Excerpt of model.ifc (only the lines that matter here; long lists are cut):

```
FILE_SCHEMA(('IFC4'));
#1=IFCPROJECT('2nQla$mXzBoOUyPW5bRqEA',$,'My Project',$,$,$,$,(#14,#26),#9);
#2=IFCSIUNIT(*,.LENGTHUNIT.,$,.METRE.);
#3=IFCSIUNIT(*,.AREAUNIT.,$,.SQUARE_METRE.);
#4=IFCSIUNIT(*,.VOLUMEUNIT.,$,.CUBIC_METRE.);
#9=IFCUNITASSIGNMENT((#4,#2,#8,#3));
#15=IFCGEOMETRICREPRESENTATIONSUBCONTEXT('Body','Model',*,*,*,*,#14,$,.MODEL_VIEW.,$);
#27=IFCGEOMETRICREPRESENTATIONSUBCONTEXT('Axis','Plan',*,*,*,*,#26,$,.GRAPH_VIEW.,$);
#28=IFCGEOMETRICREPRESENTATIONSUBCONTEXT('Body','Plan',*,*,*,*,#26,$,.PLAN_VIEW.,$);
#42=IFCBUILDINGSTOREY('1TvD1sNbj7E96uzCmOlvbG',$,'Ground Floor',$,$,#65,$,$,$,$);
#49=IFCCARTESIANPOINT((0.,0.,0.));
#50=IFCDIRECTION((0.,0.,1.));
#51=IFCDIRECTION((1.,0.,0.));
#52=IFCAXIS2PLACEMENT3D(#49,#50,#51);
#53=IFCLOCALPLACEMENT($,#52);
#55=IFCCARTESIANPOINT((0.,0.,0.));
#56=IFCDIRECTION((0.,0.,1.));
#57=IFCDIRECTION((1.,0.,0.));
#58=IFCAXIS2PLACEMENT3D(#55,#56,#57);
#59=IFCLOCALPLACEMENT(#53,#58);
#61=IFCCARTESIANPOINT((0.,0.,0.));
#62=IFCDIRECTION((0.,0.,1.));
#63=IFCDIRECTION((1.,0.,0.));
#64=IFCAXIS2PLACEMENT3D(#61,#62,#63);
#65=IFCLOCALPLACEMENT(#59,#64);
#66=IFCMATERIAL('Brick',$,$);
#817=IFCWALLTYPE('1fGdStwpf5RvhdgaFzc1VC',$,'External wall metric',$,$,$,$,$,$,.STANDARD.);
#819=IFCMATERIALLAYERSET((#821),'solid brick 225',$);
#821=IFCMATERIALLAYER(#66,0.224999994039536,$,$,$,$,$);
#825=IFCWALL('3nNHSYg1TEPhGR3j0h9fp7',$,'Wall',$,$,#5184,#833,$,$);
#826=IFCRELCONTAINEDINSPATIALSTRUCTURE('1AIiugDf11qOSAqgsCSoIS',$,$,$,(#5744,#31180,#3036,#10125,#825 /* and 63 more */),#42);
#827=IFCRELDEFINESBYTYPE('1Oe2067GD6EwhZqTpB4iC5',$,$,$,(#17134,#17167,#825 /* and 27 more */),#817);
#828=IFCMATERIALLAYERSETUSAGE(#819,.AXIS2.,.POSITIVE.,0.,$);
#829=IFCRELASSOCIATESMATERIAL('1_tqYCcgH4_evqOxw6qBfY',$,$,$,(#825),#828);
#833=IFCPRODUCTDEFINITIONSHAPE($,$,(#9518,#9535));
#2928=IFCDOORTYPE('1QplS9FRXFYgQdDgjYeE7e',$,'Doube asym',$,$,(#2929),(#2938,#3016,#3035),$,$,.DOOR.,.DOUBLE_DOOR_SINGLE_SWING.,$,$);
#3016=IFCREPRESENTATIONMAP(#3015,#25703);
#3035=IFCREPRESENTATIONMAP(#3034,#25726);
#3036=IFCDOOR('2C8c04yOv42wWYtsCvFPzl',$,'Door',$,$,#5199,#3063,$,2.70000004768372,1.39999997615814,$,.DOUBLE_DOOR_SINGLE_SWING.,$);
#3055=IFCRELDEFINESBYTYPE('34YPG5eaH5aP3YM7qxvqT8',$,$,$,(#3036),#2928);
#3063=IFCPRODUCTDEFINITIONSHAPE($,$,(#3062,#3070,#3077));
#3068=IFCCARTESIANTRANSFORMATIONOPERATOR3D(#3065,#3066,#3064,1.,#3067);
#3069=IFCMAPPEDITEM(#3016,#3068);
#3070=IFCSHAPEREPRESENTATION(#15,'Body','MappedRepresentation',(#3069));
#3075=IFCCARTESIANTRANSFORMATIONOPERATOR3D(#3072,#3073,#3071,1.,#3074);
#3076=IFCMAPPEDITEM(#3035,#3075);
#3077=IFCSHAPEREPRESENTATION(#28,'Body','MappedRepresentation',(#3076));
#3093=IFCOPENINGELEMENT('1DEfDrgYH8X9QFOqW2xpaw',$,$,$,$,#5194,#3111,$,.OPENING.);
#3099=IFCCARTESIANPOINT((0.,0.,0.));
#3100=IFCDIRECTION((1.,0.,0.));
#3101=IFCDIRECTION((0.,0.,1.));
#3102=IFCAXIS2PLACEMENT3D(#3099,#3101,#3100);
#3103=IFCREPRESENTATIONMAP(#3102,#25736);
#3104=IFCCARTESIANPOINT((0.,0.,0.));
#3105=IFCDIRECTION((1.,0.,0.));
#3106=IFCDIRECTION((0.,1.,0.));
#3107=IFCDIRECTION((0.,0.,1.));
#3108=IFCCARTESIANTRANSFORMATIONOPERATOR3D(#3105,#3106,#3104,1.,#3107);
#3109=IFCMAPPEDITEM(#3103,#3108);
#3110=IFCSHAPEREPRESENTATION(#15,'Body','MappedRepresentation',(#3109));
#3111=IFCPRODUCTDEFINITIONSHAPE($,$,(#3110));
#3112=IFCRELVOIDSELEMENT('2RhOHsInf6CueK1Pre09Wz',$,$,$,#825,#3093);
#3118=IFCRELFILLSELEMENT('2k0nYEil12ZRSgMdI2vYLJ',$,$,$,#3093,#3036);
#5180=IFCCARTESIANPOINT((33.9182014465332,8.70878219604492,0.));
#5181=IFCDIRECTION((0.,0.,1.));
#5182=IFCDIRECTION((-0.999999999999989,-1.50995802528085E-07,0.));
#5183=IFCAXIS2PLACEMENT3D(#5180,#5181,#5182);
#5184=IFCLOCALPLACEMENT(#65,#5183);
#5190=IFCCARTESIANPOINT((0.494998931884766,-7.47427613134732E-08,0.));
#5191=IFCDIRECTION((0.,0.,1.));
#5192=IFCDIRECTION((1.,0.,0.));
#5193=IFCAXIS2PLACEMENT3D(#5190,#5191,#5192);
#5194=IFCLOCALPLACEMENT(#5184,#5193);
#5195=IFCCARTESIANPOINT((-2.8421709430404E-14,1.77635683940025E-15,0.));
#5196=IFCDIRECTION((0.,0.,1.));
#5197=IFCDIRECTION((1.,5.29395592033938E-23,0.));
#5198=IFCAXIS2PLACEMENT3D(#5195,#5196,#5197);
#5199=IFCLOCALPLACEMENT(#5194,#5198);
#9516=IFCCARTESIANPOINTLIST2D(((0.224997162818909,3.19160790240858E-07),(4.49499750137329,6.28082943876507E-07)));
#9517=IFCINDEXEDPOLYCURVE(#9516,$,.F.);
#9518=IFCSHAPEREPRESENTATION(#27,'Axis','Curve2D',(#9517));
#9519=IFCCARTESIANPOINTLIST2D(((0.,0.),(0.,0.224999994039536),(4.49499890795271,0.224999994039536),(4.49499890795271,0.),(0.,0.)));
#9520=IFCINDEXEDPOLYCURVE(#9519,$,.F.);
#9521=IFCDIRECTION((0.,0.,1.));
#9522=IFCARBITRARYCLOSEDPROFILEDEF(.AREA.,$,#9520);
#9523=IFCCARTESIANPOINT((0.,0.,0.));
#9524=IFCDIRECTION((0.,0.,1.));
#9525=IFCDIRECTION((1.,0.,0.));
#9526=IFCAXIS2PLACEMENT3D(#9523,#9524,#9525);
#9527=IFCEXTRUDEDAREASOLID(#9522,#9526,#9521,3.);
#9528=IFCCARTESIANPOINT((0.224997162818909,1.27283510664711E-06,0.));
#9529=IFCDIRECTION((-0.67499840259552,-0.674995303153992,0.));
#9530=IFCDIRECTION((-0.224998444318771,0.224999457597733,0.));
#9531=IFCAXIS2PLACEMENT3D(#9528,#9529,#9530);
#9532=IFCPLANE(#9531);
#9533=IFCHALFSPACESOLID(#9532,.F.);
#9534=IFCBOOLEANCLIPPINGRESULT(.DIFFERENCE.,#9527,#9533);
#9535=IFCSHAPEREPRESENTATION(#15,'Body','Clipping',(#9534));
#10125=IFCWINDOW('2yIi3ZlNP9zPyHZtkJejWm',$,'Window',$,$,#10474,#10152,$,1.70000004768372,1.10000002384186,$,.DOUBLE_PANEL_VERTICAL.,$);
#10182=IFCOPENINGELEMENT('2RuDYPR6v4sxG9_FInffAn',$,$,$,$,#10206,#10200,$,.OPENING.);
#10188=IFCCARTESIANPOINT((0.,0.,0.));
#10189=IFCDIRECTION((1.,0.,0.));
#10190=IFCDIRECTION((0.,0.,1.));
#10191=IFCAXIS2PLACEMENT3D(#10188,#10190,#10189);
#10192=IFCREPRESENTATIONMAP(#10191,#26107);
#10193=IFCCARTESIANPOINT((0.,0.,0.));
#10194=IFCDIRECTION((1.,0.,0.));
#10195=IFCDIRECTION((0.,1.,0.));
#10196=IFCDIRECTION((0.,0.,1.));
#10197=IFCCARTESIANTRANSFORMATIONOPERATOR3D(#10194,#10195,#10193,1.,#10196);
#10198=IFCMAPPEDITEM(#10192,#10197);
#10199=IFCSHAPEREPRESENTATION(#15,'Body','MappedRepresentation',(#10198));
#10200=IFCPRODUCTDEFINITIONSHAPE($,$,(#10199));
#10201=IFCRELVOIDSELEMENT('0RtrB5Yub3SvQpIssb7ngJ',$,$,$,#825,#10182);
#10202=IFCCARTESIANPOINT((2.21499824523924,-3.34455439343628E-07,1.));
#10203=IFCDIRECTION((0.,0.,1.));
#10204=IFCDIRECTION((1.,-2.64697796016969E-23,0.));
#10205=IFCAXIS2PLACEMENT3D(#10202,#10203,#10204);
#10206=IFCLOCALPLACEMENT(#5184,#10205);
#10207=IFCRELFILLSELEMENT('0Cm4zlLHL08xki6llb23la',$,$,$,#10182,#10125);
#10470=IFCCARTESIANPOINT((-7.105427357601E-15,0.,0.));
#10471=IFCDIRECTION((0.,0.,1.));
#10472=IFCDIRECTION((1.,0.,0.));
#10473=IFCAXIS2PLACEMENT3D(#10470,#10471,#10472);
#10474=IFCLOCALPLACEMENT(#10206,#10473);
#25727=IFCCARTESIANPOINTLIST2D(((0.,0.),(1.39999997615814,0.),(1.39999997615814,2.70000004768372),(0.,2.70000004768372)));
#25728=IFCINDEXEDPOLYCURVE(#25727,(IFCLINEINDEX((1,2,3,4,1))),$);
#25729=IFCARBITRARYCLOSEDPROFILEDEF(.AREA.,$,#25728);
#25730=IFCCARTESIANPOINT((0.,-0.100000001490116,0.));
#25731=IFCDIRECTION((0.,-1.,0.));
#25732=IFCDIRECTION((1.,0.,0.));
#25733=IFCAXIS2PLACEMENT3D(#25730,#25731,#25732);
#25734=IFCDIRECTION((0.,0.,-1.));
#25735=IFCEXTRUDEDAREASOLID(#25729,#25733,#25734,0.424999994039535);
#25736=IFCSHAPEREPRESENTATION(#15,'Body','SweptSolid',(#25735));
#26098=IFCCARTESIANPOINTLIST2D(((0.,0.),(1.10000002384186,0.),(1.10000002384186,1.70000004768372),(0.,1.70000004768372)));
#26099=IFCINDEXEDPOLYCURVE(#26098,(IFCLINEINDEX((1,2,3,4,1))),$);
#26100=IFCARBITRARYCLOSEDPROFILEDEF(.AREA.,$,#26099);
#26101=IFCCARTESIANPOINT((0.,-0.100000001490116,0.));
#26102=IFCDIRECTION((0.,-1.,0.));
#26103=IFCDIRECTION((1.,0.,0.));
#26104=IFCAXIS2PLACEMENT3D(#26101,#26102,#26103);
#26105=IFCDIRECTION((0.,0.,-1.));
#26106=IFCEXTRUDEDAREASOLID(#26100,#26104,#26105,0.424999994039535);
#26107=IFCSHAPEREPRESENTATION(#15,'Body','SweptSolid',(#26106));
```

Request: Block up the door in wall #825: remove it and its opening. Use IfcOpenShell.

```python
import ifcopenshell
import ifcopenshell.api.feature
import ifcopenshell.api.root
import ifcopenshell.geom
import ifcopenshell.util.shape

model = ifcopenshell.open("model.ifc")
settings = ifcopenshell.geom.settings()


def volume(element):
    """Net volume in cubic metres, openings subtracted."""
    shape = ifcopenshell.geom.create_shape(settings, element)
    return ifcopenshell.util.shape.get_volume(shape.geometry)


door = model.by_guid("2C8c04yOv42wWYtsCvFPzl")
opening = door.FillsVoids[0].RelatingOpeningElement
wall = opening.VoidsElements[0].RelatingBuildingElement
before = volume(wall)

ifcopenshell.api.root.remove_product(model, product=door)
ifcopenshell.api.feature.remove_feature(model, feature=opening)

after = volume(wall)

print(f"wall volume {before:.3f} -> {after:.3f} m3")

model.write("model-out.ifc")
```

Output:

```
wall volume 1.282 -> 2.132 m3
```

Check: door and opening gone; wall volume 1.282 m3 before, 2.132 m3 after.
